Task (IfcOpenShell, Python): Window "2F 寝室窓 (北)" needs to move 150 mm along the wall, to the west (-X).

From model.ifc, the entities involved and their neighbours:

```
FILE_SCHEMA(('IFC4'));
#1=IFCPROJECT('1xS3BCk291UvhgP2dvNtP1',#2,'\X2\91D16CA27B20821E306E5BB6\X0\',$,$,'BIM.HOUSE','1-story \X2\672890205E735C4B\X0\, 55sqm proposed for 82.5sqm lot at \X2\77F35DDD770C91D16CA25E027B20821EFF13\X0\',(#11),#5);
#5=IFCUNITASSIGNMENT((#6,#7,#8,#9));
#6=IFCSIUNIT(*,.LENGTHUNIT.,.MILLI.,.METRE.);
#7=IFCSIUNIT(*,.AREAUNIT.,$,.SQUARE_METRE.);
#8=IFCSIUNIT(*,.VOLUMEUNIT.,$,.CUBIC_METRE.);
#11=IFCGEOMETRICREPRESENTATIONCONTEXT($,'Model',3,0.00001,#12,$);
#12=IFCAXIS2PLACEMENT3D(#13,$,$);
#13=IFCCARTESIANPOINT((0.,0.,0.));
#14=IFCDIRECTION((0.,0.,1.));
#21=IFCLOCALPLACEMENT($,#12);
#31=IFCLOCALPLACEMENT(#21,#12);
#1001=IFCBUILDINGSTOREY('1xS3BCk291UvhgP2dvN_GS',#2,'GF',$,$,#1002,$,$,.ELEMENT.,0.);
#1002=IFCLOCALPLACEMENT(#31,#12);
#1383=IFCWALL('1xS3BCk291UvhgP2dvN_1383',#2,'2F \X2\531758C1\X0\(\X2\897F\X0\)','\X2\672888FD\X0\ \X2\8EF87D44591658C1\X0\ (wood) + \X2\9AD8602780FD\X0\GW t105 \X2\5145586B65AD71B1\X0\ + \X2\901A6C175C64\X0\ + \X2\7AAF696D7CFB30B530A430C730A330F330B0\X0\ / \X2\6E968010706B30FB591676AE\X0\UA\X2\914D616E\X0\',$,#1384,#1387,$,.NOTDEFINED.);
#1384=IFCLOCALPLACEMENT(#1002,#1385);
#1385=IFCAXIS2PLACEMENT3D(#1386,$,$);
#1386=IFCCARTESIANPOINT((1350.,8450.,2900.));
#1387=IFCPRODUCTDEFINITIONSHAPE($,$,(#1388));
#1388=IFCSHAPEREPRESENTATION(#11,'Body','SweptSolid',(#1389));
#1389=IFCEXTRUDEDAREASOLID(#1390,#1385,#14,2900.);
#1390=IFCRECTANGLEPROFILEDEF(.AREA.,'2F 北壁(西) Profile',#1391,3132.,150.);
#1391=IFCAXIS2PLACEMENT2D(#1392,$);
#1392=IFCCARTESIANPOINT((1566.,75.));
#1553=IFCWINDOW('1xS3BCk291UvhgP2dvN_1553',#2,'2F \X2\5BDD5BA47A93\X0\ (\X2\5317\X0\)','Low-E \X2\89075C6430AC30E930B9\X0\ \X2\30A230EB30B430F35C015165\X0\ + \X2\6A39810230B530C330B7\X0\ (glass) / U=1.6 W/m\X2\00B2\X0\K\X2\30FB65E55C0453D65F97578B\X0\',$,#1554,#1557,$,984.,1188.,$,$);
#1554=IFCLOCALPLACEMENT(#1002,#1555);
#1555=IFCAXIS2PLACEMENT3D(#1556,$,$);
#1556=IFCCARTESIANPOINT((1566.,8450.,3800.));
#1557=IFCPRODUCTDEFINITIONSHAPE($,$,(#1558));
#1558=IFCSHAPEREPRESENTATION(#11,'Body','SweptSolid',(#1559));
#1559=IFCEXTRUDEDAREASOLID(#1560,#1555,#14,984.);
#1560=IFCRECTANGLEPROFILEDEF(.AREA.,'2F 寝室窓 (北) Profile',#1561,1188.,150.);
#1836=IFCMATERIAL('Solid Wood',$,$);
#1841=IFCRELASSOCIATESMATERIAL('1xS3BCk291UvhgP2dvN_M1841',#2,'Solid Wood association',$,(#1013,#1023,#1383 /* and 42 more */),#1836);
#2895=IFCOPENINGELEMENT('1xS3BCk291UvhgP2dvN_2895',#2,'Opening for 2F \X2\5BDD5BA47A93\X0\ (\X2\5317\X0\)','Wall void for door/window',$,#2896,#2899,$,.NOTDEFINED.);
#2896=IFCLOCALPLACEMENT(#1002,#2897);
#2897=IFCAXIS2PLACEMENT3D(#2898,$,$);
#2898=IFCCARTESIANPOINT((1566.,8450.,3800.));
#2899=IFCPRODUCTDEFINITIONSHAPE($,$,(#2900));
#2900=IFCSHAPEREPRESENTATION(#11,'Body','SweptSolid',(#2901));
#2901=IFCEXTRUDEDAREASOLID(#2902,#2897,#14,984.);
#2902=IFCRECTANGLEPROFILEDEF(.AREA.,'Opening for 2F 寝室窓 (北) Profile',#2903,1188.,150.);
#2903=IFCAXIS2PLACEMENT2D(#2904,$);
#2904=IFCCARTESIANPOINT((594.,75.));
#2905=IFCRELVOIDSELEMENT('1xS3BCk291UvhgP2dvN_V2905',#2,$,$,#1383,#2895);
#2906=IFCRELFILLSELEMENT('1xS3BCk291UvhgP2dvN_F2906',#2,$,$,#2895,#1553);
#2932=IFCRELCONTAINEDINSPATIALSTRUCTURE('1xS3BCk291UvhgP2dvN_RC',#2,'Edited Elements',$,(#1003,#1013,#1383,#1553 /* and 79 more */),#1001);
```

```python
import ifcopenshell
import ifcopenshell.api.geometry
import ifcopenshell.util.placement
import ifcopenshell.util.unit

model = ifcopenshell.open("model.ifc")
unit_scale = ifcopenshell.util.unit.calculate_unit_scale(model)

window = model.by_guid("1xS3BCk291UvhgP2dvN_1553")
opening = window.FillsVoids[0].RelatingOpeningElement
wall = opening.VoidsElements[0].RelatingBuildingElement

wall_matrix = ifcopenshell.util.placement.get_local_placement(wall.ObjectPlacement)
shift = wall_matrix[:3, 0] * -0.15 / unit_scale
before = ifcopenshell.util.placement.get_local_placement(window.ObjectPlacement)[:3, 3].copy()

# The window is not placed relative to its opening, so move both.
for product in (opening, window):
    matrix = ifcopenshell.util.placement.get_local_placement(product.ObjectPlacement)
    matrix[:3, 3] += shift
    ifcopenshell.api.geometry.edit_object_placement(model, product=product, matrix=matrix, is_si=False)

after = ifcopenshell.util.placement.get_local_placement(window.ObjectPlacement)[:3, 3]
print("window moved by", (after - before).round(3) + 0.0)

model.write("model_v2.ifc")
```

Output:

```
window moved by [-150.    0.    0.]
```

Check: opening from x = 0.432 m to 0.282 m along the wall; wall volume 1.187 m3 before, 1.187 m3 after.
